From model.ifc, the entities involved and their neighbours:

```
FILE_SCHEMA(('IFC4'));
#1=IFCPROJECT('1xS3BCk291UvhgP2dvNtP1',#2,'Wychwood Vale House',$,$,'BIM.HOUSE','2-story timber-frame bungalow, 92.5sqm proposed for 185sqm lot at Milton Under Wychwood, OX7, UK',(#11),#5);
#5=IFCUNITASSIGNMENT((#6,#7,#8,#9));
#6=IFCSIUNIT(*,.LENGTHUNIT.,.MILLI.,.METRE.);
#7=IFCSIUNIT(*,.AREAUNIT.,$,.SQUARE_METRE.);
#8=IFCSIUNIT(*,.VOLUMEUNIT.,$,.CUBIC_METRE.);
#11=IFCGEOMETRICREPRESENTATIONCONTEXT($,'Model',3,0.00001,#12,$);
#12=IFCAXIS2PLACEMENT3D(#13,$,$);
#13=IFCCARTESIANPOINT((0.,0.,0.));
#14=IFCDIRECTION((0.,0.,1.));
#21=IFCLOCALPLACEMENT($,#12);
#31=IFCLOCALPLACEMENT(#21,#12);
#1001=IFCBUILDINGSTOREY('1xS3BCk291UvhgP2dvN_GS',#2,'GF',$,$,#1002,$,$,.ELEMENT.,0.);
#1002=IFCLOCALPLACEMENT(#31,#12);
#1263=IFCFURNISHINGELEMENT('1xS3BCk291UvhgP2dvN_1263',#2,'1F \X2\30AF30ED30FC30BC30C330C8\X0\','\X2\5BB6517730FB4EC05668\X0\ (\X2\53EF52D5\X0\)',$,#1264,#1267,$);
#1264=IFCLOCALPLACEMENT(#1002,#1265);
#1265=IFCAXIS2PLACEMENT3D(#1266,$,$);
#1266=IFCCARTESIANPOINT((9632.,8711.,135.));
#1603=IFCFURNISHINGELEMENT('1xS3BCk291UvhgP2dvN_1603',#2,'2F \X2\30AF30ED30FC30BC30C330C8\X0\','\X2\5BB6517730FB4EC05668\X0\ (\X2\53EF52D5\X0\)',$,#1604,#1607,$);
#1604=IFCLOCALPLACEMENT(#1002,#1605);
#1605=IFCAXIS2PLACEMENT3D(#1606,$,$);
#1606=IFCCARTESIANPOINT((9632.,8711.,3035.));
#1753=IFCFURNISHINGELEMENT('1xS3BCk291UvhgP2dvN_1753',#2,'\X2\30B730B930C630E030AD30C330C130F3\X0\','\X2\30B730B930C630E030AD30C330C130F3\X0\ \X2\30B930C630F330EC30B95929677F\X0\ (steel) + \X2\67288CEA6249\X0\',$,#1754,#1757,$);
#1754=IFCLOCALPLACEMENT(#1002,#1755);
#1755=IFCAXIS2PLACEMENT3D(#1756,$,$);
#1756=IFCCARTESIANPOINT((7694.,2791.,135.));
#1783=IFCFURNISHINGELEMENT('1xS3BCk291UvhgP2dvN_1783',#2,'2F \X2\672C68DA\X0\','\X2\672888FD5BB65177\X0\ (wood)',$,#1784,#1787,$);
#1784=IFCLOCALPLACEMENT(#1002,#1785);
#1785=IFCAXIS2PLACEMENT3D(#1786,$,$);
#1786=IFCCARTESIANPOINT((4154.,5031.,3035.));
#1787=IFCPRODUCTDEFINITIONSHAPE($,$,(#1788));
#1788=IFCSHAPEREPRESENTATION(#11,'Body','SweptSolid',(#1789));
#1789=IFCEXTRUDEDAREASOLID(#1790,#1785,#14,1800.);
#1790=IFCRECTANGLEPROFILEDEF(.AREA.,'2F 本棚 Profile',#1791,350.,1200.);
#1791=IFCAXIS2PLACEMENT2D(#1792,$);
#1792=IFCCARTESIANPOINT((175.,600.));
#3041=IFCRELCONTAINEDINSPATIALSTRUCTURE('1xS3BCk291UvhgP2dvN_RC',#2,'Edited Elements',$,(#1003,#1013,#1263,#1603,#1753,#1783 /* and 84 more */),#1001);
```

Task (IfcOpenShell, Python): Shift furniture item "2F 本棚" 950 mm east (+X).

```python
import ifcopenshell
import ifcopenshell.api.geometry
import ifcopenshell.util.placement
import ifcopenshell.util.unit

model = ifcopenshell.open("model.ifc")
unit_scale = ifcopenshell.util.unit.calculate_unit_scale(model)

item = model.by_guid("1xS3BCk291UvhgP2dvN_1783")
matrix = ifcopenshell.util.placement.get_local_placement(item.ObjectPlacement)
matrix[0, 3] += 0.95 / unit_scale
ifcopenshell.api.geometry.edit_object_placement(model, product=item, matrix=matrix, is_si=False)

print(ifcopenshell.util.placement.get_local_placement(item.ObjectPlacement).round(3) + 0.0)

model.write("model_updated.ifc")
```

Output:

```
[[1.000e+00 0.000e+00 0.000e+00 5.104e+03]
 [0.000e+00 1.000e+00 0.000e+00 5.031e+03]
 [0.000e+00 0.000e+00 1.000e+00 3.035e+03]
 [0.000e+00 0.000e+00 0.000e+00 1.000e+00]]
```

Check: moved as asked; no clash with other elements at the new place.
